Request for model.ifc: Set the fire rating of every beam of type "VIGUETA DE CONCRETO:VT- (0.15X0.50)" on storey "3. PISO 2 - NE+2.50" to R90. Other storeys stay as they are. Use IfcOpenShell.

First a look at what the model holds.

```python
import ifcopenshell
import ifcopenshell.util.element

model = ifcopenshell.open("model.ifc")
print(model.schema)
storey = next(s for s in model.by_type("IfcBuildingStorey") if s.Name == "3. PISO 2 - NE+2.50")
beams = [e for e in ifcopenshell.util.element.get_decomposition(storey) if e.is_a("IfcBeam")]
seen = {}
for e in beams:
    element_type = ifcopenshell.util.element.get_type(e)
    key = (element_type.Name if element_type != e and element_type else None, ifcopenshell.util.element.get_pset(e, "Pset_BeamCommon", "FireRating"))
    seen[key] = seen.get(key, 0) + 1
for (name, value), count in sorted(seen.items(), key=str):
    print(count, "x", name, "|", value)
```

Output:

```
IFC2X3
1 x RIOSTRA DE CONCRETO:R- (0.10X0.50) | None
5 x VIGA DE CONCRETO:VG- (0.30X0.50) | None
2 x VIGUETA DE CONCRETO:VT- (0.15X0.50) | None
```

```python
import ifcopenshell
import ifcopenshell.api.pset
import ifcopenshell.util.element

model = ifcopenshell.open("model.ifc")

storey = next(s for s in model.by_type("IfcBuildingStorey") if s.Name == "3. PISO 2 - NE+2.50")
beams = [e for e in ifcopenshell.util.element.get_decomposition(storey) if e.is_a("IfcBeam")]

count = 0
for e in beams:
    element_type = ifcopenshell.util.element.get_type(e)
    if element_type in (None, e) or element_type.Name != "VIGUETA DE CONCRETO:VT- (0.15X0.50)":
        continue
    # add_pset returns the element's existing set when there is one.
    pset = ifcopenshell.api.pset.add_pset(model, product=e, name="Pset_BeamCommon")
    ifcopenshell.api.pset.edit_pset(model, pset=pset, properties={"FireRating": "R90"})
    count += 1

print(count, "beams updated")

model.write("model_v2.ifc")
```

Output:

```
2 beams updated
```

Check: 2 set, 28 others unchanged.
